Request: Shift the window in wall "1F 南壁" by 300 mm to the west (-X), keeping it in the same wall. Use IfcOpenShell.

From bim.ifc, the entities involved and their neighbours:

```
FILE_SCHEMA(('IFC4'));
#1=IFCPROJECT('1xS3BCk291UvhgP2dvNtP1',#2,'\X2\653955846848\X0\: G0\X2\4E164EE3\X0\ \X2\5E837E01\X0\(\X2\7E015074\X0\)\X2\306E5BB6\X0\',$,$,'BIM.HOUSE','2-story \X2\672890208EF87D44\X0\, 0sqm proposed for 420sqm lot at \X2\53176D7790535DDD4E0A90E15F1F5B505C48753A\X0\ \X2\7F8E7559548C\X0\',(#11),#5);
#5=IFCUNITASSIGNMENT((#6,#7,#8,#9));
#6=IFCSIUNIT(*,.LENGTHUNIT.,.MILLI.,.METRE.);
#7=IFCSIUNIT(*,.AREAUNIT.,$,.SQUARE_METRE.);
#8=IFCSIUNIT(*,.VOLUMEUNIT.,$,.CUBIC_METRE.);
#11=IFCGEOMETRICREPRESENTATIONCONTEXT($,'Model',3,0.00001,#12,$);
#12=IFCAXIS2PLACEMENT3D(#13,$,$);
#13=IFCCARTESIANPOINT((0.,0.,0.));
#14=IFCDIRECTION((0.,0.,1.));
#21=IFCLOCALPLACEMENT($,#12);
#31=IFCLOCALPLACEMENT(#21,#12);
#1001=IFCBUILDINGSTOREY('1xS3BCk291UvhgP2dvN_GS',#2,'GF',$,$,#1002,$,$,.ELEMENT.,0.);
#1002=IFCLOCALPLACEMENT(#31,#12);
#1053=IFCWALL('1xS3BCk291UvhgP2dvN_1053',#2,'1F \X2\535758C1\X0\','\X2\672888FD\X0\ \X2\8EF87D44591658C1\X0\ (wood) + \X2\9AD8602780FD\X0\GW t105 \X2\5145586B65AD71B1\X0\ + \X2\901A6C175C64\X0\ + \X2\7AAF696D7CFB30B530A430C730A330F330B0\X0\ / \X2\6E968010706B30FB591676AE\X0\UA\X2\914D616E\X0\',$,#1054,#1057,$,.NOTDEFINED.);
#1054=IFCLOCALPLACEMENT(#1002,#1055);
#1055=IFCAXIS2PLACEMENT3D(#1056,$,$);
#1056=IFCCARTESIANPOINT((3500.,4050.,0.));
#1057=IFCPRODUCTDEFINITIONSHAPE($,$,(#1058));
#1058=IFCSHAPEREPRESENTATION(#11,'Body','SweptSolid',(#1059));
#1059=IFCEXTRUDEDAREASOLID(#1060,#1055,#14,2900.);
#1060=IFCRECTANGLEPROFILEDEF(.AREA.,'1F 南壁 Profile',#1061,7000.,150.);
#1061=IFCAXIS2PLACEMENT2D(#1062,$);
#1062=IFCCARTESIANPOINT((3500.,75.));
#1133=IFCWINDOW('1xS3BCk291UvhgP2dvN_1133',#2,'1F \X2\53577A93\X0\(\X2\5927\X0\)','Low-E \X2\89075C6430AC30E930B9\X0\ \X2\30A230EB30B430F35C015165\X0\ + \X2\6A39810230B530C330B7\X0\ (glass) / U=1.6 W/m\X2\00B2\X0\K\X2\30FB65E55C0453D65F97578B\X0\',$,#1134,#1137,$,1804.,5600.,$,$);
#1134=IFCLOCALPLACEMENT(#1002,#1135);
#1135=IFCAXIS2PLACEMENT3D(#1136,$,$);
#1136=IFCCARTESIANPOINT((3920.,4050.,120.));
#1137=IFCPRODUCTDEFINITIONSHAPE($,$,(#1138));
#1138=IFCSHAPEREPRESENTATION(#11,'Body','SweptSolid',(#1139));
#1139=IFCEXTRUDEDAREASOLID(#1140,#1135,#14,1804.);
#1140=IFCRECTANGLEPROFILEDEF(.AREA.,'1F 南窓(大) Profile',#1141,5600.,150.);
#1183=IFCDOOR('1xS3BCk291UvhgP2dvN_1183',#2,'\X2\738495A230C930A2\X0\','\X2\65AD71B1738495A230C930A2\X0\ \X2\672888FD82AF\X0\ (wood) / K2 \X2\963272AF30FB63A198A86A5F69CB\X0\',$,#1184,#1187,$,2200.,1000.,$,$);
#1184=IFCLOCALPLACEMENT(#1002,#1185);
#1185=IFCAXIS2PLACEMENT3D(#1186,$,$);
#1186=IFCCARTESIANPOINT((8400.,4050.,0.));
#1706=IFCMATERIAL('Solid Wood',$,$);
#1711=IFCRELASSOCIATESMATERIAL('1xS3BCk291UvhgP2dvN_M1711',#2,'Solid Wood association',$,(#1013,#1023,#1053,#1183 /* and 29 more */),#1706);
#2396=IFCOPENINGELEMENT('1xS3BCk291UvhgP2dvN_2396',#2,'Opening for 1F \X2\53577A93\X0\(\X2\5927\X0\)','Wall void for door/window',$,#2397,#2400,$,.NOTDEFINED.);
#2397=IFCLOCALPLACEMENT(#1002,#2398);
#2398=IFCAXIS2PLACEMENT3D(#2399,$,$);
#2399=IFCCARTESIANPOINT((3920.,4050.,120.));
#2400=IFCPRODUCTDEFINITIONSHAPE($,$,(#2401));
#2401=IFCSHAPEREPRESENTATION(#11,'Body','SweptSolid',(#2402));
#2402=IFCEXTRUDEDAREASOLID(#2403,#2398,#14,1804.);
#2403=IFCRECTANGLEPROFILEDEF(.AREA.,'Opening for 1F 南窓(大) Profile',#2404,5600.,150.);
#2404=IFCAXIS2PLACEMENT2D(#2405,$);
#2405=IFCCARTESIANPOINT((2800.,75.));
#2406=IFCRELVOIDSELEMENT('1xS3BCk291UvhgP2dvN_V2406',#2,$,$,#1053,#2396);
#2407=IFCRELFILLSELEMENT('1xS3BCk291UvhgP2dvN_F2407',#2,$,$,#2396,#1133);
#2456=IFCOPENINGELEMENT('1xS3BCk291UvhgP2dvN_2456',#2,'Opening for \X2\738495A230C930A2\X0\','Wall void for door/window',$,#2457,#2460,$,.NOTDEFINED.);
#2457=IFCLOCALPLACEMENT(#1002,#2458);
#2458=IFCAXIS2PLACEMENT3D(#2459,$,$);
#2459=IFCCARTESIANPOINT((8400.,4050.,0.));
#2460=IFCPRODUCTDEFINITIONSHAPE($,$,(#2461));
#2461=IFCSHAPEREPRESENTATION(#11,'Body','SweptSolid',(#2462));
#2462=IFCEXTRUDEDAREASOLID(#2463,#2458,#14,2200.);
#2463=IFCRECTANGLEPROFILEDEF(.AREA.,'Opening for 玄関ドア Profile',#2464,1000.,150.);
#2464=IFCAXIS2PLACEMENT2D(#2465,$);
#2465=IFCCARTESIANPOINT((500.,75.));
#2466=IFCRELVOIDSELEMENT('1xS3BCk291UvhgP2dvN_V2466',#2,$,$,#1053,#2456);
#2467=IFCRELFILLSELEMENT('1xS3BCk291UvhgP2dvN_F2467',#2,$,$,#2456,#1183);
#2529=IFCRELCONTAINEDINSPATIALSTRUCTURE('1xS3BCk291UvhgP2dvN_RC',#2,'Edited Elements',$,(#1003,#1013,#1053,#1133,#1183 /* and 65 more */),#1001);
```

```python
import ifcopenshell
import ifcopenshell.api.geometry
import ifcopenshell.util.placement
import ifcopenshell.util.unit

model = ifcopenshell.open("bim.ifc")
unit_scale = ifcopenshell.util.unit.calculate_unit_scale(model)

window = model.by_id(1133)
opening = window.FillsVoids[0].RelatingOpeningElement
wall = opening.VoidsElements[0].RelatingBuildingElement

wall_matrix = ifcopenshell.util.placement.get_local_placement(wall.ObjectPlacement)
shift = wall_matrix[:3, 0] * -0.3 / unit_scale
before = ifcopenshell.util.placement.get_local_placement(window.ObjectPlacement)[:3, 3].copy()

# The window is not placed relative to its opening, so move both.
for product in (opening, window):
    matrix = ifcopenshell.util.placement.get_local_placement(product.ObjectPlacement)
    matrix[:3, 3] += shift
    ifcopenshell.api.geometry.edit_object_placement(model, product=product, matrix=matrix, is_si=False)

after = ifcopenshell.util.placement.get_local_placement(window.ObjectPlacement)[:3, 3]
print("window moved by", (after - before).round(3) + 0.0)

model.write("bim_edited.ifc")
```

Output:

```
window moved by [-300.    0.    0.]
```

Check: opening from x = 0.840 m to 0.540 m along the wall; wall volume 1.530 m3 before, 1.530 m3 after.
